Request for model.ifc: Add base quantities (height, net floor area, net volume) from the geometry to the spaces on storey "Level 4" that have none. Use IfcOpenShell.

First a look at what the model holds.

```python
import ifcopenshell
import ifcopenshell.util.element
import ifcopenshell.util.unit

model = ifcopenshell.open("model.ifc")
print(model.schema)
for unit_type in ("LENGTHUNIT", "AREAUNIT", "VOLUMEUNIT"):
    print(unit_type, ifcopenshell.util.unit.calculate_unit_scale(model, unit_type))
storey = next(s for s in model.by_type("IfcBuildingStorey") if s.Name == "Level 4")
spaces = [e for e in ifcopenshell.util.element.get_decomposition(storey) if e.is_a("IfcSpace")]
for e in sorted(spaces, key=lambda e: e.id()):
    print(e.id(), e.is_a(), e.Name, list(ifcopenshell.util.element.get_psets(e, qtos_only=True)), sep=" | ")
```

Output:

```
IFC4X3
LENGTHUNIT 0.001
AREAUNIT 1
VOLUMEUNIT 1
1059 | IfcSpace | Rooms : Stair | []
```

```python
import ifcopenshell
import ifcopenshell.api.pset
import ifcopenshell.geom
import ifcopenshell.util.element
import ifcopenshell.util.shape
import ifcopenshell.util.unit

model = ifcopenshell.open("model.ifc")
unit_scale = ifcopenshell.util.unit.calculate_unit_scale(model)
area_scale = ifcopenshell.util.unit.calculate_unit_scale(model, "AREAUNIT")
volume_scale = ifcopenshell.util.unit.calculate_unit_scale(model, "VOLUMEUNIT")
settings = ifcopenshell.geom.settings()

storey = next(s for s in model.by_type("IfcBuildingStorey") if s.Name == "Level 4")
spaces = [e for e in ifcopenshell.util.element.get_decomposition(storey) if e.is_a("IfcSpace")]

for e in sorted(spaces, key=lambda e: e.id()):
    if ifcopenshell.util.element.get_psets(e, qtos_only=True, should_inherit=False):
        continue
    # Geometry comes back in metres, in the element's own axes.
    shape = ifcopenshell.geom.create_shape(settings, e)
    values = {
        "Height": ifcopenshell.util.shape.get_z(shape.geometry) / unit_scale,
        "NetFloorArea": ifcopenshell.util.shape.get_footprint_area(shape.geometry) / area_scale,
        "NetVolume": ifcopenshell.util.shape.get_volume(shape.geometry) / volume_scale,
    }
    qto = ifcopenshell.api.pset.add_qto(model, product=e, name="Qto_SpaceBaseQuantities")
    ifcopenshell.api.pset.edit_qto(model, qto=qto, properties=values)
    print(e.id(), {k: round(v, 3) for k, v in values.items()})

model.write("model_edited.ifc")
```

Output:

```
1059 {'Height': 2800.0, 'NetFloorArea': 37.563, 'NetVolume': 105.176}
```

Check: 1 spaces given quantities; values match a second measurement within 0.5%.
